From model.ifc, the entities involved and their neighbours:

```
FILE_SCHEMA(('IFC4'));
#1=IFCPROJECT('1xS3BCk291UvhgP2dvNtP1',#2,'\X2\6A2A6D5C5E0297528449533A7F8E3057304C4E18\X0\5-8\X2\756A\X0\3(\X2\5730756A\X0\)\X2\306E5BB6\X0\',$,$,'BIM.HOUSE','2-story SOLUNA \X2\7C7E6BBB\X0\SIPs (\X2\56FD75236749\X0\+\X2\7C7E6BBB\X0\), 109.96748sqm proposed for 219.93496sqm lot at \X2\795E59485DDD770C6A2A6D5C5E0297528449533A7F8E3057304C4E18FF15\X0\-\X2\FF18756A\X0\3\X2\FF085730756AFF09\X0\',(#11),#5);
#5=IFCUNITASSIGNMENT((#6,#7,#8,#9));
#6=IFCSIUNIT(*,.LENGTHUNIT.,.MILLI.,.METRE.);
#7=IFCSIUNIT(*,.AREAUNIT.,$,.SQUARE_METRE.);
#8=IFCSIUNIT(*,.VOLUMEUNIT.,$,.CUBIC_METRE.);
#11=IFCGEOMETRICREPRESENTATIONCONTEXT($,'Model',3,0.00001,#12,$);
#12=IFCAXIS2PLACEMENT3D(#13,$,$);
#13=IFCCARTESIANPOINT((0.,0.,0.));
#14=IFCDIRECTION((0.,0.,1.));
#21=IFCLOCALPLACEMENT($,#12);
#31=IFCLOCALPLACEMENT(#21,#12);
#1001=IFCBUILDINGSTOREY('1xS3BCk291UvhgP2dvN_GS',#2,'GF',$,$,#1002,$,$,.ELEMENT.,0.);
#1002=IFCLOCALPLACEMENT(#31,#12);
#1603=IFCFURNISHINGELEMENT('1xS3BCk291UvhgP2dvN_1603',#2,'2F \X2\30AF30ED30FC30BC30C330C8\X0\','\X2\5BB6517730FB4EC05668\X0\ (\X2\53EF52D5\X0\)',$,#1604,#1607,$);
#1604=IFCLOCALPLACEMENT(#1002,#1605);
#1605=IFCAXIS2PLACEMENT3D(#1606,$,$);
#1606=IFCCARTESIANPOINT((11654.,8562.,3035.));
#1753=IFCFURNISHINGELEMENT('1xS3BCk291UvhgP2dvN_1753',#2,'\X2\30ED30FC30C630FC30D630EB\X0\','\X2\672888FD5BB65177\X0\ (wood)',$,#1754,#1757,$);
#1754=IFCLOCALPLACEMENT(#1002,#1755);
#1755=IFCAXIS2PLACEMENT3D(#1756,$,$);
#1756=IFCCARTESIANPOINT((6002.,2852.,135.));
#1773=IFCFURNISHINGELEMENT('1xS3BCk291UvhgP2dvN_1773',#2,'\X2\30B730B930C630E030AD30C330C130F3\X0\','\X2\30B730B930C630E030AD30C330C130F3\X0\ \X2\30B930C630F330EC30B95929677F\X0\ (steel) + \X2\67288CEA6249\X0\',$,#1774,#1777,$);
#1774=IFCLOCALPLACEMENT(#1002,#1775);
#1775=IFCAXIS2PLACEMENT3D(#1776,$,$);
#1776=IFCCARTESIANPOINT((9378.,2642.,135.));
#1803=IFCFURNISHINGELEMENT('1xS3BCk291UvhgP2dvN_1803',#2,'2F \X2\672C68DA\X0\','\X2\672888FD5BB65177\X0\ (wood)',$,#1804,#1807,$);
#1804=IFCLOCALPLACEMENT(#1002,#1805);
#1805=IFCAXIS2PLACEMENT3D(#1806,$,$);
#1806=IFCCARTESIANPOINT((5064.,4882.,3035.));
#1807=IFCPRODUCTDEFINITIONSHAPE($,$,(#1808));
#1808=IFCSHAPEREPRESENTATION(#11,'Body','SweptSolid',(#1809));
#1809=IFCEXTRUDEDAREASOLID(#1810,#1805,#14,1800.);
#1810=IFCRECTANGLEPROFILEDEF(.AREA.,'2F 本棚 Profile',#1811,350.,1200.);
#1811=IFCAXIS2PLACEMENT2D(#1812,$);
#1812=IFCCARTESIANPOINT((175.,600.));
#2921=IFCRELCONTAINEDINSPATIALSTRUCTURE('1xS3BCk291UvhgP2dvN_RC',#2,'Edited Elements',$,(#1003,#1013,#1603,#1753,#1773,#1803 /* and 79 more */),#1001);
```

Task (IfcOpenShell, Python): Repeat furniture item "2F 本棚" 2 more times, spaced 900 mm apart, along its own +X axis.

```python
import ifcopenshell
import ifcopenshell.api.geometry
import ifcopenshell.api.root
import ifcopenshell.util.element
import ifcopenshell.util.placement
import ifcopenshell.util.unit

model = ifcopenshell.open("model.ifc")
unit_scale = ifcopenshell.util.unit.calculate_unit_scale(model)


def reuse_history(source, copy):
    """copy_class also copies each property set's owner history, people and application; keep the originals."""
    for rel in copy.IsDefinedBy:
        if rel.is_a("IfcRelDefinesByProperties") and (history := rel.RelatingPropertyDefinition.OwnerHistory):
            rel.RelatingPropertyDefinition.OwnerHistory = source.OwnerHistory
            ifcopenshell.util.element.remove_deep2(model, history)


source = model.by_guid("1xS3BCk291UvhgP2dvN_1803")
base = ifcopenshell.util.placement.get_local_placement(source.ObjectPlacement)
step = base[:3, 0] * 0.9 / unit_scale

for i in range(1, 3):
    copy = ifcopenshell.api.root.copy_class(model, product=source)
    copy.Representation = ifcopenshell.util.element.copy_deep(
        model, source.Representation, exclude=["IfcGeometricRepresentationContext", "IfcRepresentationMap"]
    )
    reuse_history(source, copy)
    matrix = base.copy()
    matrix[:3, 3] += i * step
    print("added at", matrix[:3, 3].round(3) + 0.0)
    ifcopenshell.api.geometry.edit_object_placement(model, product=copy, matrix=matrix, is_si=False)

model.write("model_rev.ifc")
```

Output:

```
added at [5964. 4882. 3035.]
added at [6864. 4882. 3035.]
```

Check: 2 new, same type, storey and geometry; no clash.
